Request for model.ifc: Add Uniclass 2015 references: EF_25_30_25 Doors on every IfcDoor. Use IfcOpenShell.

First a look at what the model holds.

```python
import ifcopenshell

model = ifcopenshell.open("model.ifc")
print(model.schema)
print("classifications:", [c.Name for c in model.by_type("IfcClassification")])
for ifc_class in ("IfcDoor", "IfcRoof", "IfcStair", "IfcWall", "IfcWindow"):
    print(ifc_class, len(model.by_type(ifc_class)))
```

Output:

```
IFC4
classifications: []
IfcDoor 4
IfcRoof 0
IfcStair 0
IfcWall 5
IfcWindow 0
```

```python
import ifcopenshell
import ifcopenshell.api.classification

model = ifcopenshell.open("model.ifc")

system = ifcopenshell.api.classification.add_classification(model, classification="Uniclass 2015")

codes = {
    "IfcDoor": ("EF_25_30_25", "Doors"),
}
for ifc_class, (code, name) in codes.items():
    products = model.by_type(ifc_class)
    ifcopenshell.api.classification.add_reference(
        model, products=products, classification=system, identification=code, name=name
    )
    print(code, len(products))

model.write("model_v2.ifc")
```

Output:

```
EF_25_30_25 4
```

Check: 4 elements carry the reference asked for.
